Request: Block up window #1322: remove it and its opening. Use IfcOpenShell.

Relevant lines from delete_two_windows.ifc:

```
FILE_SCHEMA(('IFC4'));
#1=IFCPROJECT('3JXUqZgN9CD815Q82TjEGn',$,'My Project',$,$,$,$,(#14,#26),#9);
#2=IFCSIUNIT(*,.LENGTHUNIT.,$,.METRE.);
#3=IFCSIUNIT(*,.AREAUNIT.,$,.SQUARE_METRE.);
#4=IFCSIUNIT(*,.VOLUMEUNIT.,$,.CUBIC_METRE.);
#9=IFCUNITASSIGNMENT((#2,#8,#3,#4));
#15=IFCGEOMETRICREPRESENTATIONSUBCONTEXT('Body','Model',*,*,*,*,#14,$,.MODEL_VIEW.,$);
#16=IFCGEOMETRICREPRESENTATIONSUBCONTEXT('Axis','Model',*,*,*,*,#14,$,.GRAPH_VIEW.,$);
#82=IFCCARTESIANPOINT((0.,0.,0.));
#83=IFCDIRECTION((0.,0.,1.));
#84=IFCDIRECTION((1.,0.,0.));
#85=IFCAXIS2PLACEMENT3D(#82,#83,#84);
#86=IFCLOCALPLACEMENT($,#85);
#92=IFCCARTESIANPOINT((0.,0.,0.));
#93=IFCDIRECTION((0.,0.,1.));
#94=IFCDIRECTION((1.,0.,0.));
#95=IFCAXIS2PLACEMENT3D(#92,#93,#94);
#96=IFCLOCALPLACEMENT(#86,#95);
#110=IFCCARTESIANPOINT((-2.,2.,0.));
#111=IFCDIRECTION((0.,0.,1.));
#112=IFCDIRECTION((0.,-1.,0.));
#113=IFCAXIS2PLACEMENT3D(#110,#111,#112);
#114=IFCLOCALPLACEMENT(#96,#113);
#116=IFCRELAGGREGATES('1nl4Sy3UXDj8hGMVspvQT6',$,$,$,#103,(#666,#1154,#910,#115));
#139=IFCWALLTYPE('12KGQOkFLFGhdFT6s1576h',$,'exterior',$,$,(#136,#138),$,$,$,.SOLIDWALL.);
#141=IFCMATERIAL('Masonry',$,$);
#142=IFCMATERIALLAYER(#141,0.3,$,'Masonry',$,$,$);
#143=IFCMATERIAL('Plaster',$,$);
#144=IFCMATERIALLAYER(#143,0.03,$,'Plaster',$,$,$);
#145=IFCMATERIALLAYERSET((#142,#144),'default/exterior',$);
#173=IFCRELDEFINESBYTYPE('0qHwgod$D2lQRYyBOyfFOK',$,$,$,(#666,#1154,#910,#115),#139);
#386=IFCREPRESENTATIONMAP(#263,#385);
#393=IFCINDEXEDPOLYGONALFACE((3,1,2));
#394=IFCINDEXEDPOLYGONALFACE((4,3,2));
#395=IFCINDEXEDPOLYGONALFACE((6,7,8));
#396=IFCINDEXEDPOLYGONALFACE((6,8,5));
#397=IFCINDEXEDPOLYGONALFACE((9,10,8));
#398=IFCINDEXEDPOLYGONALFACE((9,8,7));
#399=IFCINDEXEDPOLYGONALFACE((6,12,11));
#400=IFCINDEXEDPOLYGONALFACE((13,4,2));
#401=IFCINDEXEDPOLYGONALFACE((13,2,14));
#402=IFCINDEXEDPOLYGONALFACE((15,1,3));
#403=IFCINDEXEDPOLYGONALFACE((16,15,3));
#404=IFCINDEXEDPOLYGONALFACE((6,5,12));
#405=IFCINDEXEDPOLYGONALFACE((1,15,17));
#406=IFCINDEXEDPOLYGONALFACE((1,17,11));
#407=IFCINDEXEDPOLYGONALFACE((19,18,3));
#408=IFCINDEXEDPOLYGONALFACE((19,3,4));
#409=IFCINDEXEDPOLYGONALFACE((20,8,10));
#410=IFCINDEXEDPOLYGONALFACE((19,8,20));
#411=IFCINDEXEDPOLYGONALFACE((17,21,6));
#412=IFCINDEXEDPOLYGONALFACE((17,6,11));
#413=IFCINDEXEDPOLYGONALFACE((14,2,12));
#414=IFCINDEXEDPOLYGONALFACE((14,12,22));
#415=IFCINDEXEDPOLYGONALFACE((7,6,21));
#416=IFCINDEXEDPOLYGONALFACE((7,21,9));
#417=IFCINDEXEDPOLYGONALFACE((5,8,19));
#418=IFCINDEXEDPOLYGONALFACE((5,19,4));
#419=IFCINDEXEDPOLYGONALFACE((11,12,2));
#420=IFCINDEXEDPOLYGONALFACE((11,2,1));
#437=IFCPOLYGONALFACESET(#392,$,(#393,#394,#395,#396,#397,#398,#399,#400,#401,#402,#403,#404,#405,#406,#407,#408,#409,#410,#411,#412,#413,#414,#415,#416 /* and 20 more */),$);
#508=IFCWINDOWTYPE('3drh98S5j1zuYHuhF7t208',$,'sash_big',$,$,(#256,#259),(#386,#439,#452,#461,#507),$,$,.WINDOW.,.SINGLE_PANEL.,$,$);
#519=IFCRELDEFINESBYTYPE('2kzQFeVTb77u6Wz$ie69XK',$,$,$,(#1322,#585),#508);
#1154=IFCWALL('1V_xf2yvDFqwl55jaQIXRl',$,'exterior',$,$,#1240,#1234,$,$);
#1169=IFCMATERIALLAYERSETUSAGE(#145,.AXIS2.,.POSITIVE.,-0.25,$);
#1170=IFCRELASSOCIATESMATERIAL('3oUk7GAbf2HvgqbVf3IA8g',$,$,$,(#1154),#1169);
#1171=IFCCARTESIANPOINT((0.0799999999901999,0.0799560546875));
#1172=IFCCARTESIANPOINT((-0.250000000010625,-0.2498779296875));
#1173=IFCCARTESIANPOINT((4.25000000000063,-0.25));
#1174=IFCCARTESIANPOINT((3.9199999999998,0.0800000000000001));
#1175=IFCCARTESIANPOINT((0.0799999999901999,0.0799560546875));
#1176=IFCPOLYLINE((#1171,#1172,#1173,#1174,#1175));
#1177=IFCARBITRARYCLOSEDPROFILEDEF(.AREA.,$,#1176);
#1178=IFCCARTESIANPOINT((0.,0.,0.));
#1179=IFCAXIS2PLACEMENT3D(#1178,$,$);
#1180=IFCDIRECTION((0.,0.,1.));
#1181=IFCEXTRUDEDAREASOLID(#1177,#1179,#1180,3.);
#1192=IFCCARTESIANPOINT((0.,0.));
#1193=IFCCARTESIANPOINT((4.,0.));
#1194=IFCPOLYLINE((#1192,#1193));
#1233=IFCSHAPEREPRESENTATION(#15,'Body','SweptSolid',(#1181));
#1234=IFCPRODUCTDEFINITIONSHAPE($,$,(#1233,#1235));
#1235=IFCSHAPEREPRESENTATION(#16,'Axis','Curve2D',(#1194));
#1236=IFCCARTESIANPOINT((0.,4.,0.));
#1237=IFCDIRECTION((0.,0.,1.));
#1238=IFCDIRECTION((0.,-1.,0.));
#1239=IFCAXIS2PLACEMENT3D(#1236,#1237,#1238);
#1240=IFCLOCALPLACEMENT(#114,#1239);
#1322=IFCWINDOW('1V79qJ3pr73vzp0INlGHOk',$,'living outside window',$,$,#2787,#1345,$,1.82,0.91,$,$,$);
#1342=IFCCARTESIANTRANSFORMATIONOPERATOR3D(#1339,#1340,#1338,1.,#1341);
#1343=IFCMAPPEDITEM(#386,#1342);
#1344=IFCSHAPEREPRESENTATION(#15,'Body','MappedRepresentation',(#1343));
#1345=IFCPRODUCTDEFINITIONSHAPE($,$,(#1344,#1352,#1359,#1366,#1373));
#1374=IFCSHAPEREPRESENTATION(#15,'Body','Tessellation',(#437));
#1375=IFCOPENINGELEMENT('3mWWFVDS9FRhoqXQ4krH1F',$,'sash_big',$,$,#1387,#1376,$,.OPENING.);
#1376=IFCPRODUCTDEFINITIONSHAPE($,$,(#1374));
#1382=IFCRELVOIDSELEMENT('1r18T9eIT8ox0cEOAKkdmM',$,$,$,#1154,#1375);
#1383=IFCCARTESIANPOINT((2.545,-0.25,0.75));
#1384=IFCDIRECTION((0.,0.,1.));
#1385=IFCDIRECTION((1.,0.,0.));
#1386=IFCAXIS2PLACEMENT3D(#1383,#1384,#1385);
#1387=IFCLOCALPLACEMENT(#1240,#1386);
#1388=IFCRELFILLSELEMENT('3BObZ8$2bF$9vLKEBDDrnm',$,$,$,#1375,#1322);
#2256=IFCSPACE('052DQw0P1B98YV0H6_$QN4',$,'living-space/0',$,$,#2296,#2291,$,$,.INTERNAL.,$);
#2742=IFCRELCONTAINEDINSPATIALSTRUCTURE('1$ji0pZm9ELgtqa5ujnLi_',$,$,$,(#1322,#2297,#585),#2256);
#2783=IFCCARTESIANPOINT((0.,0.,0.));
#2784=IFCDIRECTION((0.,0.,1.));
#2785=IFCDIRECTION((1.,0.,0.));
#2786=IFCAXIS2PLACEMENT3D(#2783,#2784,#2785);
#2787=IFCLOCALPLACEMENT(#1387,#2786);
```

```python
import ifcopenshell
import ifcopenshell.api.feature
import ifcopenshell.api.root
import ifcopenshell.geom
import ifcopenshell.util.shape

model = ifcopenshell.open("delete_two_windows.ifc")
settings = ifcopenshell.geom.settings()


def volume(element):
    """Net volume in cubic metres, openings subtracted."""
    shape = ifcopenshell.geom.create_shape(settings, element)
    return ifcopenshell.util.shape.get_volume(shape.geometry)


window = model.by_guid("1V79qJ3pr73vzp0INlGHOk")
opening = window.FillsVoids[0].RelatingOpeningElement
wall = opening.VoidsElements[0].RelatingBuildingElement
before = volume(wall)

ifcopenshell.api.root.remove_product(model, product=window)
ifcopenshell.api.feature.remove_feature(model, feature=opening)

after = volume(wall)

print(f"wall volume {before:.3f} -> {after:.3f} m3")

model.write("delete_two_windows_v2.ifc")
```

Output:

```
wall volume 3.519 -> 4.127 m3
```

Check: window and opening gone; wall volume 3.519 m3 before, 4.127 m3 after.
